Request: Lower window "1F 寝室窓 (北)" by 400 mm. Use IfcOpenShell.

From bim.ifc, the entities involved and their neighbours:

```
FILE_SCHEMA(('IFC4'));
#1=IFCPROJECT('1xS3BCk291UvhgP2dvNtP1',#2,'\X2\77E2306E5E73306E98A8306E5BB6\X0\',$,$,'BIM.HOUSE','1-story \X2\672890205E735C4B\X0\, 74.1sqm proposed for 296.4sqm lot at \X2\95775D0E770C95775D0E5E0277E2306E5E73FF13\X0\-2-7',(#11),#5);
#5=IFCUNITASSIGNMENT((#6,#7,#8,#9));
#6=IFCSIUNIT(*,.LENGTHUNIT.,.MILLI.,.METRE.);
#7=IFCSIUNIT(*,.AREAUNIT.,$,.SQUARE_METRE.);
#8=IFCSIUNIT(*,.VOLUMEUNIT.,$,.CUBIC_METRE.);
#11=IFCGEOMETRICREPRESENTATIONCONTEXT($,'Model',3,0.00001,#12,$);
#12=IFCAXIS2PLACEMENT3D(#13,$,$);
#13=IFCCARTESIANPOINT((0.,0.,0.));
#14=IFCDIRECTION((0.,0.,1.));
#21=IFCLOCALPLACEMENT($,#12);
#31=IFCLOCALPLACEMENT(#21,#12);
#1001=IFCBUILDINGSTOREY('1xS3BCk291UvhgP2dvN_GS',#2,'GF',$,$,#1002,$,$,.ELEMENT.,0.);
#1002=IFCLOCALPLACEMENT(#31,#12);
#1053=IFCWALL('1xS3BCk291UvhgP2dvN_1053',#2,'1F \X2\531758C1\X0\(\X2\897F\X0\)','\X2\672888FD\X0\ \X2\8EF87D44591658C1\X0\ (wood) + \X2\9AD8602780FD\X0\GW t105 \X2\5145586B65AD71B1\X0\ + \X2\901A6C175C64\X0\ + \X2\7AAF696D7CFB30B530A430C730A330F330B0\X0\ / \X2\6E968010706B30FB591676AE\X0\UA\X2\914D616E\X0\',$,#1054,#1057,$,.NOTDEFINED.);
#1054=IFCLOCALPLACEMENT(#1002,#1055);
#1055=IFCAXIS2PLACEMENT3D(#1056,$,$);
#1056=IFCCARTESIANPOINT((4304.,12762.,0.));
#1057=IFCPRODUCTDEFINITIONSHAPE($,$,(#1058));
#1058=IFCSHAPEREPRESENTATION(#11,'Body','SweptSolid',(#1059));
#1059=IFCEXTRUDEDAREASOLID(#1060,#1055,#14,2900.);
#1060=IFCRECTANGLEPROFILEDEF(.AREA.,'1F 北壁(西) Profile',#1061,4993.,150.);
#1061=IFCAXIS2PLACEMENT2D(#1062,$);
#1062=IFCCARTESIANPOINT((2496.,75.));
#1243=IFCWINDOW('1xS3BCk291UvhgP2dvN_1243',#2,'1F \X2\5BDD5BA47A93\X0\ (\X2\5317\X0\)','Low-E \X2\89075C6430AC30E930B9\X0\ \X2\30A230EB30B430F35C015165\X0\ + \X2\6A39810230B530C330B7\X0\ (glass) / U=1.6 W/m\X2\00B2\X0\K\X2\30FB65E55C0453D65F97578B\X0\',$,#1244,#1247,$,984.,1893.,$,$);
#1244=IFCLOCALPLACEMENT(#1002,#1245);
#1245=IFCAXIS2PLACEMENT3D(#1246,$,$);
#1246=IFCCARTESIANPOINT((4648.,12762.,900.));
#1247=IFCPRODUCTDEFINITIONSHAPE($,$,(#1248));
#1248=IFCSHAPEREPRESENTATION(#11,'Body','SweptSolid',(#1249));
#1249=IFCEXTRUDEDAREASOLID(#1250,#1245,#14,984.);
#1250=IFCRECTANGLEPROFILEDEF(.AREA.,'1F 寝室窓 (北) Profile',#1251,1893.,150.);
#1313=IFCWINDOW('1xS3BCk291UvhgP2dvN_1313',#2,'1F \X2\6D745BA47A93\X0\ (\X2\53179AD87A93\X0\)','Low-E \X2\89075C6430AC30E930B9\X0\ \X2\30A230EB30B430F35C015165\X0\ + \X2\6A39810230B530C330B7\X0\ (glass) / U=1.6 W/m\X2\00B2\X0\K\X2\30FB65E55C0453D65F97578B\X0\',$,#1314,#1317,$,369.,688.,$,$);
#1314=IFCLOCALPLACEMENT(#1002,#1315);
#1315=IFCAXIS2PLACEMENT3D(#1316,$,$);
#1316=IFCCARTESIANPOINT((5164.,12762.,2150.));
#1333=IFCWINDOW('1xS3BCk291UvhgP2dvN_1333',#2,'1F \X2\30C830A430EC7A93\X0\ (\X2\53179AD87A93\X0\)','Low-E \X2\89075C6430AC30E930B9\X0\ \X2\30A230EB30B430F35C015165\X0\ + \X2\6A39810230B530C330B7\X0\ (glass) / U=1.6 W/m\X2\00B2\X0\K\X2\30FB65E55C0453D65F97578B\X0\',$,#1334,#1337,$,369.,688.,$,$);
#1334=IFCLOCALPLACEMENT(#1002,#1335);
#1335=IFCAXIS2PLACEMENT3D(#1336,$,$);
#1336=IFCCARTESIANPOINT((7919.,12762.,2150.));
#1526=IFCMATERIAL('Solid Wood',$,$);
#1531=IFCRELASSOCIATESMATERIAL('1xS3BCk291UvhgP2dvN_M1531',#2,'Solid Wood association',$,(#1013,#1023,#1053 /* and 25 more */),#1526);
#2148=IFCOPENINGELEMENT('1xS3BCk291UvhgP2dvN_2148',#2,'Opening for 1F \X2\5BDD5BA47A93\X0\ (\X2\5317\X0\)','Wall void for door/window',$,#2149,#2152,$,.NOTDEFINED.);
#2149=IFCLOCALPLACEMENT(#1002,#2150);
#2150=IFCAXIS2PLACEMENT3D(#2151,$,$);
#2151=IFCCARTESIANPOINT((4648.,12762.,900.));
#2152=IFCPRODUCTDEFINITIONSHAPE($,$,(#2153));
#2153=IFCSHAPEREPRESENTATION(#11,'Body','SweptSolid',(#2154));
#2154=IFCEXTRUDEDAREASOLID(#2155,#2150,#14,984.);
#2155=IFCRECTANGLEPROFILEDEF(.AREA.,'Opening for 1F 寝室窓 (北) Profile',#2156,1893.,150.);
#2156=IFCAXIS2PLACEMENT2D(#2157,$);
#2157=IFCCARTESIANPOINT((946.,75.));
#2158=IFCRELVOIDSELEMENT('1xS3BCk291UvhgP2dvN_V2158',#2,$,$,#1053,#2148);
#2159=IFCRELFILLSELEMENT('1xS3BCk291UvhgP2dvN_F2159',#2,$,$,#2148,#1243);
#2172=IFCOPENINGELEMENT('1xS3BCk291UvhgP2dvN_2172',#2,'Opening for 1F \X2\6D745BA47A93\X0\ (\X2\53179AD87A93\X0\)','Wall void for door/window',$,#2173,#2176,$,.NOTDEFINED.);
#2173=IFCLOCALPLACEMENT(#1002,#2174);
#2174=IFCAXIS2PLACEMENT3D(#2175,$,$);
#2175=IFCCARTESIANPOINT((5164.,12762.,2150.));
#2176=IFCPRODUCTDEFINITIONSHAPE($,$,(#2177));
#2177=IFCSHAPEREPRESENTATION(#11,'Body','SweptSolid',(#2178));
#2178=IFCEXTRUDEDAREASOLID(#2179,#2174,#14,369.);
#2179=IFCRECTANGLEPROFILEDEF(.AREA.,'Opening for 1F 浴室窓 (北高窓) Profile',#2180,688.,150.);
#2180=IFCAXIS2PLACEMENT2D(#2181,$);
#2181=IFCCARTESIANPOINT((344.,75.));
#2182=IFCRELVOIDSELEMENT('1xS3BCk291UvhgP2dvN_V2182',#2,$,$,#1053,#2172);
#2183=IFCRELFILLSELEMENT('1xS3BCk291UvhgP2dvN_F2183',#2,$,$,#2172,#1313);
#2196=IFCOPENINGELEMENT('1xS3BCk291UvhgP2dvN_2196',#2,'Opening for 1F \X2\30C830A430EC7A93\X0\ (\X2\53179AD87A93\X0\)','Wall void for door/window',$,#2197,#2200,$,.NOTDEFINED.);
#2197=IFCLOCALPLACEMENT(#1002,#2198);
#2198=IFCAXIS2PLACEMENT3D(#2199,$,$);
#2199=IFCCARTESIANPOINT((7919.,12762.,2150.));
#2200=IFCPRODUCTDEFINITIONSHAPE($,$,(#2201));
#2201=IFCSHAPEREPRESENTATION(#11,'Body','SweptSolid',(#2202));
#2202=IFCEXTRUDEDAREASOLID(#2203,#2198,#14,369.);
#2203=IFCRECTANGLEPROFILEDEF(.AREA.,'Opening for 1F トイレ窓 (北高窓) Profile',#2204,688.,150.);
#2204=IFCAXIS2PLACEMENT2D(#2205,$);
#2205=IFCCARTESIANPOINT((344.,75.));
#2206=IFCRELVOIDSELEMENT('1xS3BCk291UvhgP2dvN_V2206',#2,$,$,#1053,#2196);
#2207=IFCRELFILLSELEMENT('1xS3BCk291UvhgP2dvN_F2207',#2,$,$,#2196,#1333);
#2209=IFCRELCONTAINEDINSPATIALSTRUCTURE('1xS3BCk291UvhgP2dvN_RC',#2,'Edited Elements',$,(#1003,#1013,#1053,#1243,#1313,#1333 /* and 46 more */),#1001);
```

```python
import numpy as np
import ifcopenshell
import ifcopenshell.api.geometry
import ifcopenshell.util.placement
import ifcopenshell.util.unit

model = ifcopenshell.open("bim.ifc")
unit_scale = ifcopenshell.util.unit.calculate_unit_scale(model)

window = model.by_id(1243)
opening = window.FillsVoids[0].RelatingOpeningElement
dz = -0.4 / unit_scale

shift = np.array([0.0, 0.0, dz])
# The window is not placed relative to its opening, so move both.
for product in (opening, window):
    matrix = ifcopenshell.util.placement.get_local_placement(product.ObjectPlacement)
    matrix[:3, 3] += shift
    ifcopenshell.api.geometry.edit_object_placement(model, product=product, matrix=matrix, is_si=False)

print(f"moved by {dz * unit_scale:+.3f} m")

model.write("bim_updated.ifc")
```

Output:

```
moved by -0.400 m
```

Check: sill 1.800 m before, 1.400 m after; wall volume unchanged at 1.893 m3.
